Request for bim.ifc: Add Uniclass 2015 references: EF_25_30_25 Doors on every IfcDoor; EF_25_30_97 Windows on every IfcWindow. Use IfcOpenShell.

First a look at what the model holds.

```python
import ifcopenshell

model = ifcopenshell.open("bim.ifc")
print(model.schema)
print("classifications:", [c.Name for c in model.by_type("IfcClassification")])
for ifc_class in ("IfcDoor", "IfcRoof", "IfcStair", "IfcWall", "IfcWindow"):
    print(ifc_class, len(model.by_type(ifc_class)))
```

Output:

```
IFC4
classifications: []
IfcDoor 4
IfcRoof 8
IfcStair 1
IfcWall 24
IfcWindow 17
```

```python
import ifcopenshell
import ifcopenshell.api.classification

model = ifcopenshell.open("bim.ifc")

system = ifcopenshell.api.classification.add_classification(model, classification="Uniclass 2015")

codes = {
    "IfcDoor": ("EF_25_30_25", "Doors"),
    "IfcWindow": ("EF_25_30_97", "Windows"),
}
for ifc_class, (code, name) in codes.items():
    products = model.by_type(ifc_class)
    ifcopenshell.api.classification.add_reference(
        model, products=products, classification=system, identification=code, name=name
    )
    print(code, len(products))

model.write("bim_edited.ifc")
```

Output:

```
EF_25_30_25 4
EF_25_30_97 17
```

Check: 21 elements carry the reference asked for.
